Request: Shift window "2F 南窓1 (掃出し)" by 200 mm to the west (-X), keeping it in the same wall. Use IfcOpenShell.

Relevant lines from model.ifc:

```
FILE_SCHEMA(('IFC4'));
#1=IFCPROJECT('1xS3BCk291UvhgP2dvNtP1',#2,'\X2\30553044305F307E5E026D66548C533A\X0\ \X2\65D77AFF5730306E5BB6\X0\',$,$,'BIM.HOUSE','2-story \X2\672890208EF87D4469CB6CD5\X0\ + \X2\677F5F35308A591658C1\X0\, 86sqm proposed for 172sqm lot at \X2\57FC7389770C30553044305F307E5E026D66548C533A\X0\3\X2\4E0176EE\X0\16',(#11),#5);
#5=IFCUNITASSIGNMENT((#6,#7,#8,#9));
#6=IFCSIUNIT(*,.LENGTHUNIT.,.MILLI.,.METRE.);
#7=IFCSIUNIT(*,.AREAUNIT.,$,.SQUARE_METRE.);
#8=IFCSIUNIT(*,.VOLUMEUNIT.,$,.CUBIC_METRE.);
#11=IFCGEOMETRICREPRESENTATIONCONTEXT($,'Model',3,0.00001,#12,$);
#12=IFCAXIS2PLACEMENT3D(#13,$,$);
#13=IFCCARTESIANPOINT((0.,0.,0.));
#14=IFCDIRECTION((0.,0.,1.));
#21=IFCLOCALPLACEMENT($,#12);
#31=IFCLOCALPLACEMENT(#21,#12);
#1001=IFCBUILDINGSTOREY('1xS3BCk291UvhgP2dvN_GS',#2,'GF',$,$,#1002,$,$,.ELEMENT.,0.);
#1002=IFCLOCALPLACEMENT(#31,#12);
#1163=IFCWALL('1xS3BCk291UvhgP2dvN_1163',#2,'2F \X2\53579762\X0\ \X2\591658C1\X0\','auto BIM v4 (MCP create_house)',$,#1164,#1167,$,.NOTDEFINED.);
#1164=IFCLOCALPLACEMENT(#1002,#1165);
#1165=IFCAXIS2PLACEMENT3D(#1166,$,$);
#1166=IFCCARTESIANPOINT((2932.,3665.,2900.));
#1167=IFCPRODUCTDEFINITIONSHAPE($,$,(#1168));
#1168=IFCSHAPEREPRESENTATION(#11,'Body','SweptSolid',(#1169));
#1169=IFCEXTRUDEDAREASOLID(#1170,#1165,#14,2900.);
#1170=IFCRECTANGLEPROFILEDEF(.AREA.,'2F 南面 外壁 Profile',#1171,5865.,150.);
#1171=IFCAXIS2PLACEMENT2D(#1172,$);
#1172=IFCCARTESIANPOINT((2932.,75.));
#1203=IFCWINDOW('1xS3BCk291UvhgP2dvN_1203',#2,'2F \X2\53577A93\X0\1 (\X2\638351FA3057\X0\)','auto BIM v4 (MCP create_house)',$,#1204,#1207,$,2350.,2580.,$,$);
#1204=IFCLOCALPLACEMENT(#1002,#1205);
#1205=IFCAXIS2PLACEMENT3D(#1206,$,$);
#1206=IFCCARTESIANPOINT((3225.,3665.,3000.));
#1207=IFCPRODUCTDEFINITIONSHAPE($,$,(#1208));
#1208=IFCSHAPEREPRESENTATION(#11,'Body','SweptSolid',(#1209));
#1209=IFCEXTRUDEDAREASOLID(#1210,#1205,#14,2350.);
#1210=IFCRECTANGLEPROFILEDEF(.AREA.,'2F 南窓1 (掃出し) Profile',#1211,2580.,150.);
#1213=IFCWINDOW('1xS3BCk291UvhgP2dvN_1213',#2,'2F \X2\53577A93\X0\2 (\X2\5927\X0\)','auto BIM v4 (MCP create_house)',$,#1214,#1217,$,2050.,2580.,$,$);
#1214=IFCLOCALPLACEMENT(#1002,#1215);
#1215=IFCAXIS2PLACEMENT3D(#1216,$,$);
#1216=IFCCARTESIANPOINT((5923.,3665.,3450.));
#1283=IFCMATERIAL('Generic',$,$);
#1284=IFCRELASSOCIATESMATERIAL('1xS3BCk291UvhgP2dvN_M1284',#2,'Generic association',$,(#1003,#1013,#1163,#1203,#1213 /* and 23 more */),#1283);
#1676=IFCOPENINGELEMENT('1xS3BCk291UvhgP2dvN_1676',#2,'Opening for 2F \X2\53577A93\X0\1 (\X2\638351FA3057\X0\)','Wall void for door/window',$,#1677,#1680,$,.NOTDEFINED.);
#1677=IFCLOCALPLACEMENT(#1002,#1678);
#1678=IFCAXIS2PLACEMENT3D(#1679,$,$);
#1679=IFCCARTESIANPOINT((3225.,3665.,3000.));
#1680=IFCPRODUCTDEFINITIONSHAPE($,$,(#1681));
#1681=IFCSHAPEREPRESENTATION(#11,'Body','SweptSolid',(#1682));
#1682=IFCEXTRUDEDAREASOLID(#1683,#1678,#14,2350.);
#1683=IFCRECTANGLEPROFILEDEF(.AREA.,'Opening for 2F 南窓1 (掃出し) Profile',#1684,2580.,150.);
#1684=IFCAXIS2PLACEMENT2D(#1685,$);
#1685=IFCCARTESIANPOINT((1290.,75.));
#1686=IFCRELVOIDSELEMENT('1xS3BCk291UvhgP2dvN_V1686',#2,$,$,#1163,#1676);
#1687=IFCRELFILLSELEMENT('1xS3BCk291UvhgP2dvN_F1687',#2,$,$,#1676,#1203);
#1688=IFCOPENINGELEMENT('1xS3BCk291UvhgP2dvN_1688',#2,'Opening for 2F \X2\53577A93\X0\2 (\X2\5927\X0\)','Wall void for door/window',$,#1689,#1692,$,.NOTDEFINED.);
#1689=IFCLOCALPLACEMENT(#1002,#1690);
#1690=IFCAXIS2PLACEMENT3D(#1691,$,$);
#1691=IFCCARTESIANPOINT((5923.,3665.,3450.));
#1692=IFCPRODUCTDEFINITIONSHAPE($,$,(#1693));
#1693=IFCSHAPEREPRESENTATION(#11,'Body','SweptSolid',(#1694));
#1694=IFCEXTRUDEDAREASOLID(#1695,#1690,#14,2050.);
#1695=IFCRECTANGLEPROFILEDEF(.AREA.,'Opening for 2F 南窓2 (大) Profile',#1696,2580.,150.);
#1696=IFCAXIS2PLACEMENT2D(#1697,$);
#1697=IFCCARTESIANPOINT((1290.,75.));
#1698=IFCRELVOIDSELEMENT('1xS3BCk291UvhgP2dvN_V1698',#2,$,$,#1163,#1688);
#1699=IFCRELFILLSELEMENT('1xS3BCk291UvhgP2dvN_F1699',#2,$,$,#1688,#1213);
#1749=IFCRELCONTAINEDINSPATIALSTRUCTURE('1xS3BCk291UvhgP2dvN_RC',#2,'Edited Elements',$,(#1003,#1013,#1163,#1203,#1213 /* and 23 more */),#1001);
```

```python
import ifcopenshell
import ifcopenshell.api.geometry
import ifcopenshell.util.placement
import ifcopenshell.util.unit

model = ifcopenshell.open("model.ifc")
unit_scale = ifcopenshell.util.unit.calculate_unit_scale(model)

window = model.by_guid("1xS3BCk291UvhgP2dvN_1203")
opening = window.FillsVoids[0].RelatingOpeningElement
wall = opening.VoidsElements[0].RelatingBuildingElement

wall_matrix = ifcopenshell.util.placement.get_local_placement(wall.ObjectPlacement)
shift = wall_matrix[:3, 0] * -0.2 / unit_scale
before = ifcopenshell.util.placement.get_local_placement(window.ObjectPlacement)[:3, 3].copy()

# The window is not placed relative to its opening, so move both.
for product in (opening, window):
    matrix = ifcopenshell.util.placement.get_local_placement(product.ObjectPlacement)
    matrix[:3, 3] += shift
    ifcopenshell.api.geometry.edit_object_placement(model, product=product, matrix=matrix, is_si=False)

after = ifcopenshell.util.placement.get_local_placement(window.ObjectPlacement)[:3, 3]
print("window moved by", (after - before).round(3) + 0.0)

model.write("model_rev.ifc")
```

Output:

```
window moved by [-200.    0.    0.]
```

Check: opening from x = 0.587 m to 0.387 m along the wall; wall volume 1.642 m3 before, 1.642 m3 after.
